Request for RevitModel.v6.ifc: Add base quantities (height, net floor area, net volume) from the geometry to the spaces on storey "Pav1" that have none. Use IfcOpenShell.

First a look at what the model holds.

```python
import ifcopenshell
import ifcopenshell.util.element
import ifcopenshell.util.unit

model = ifcopenshell.open("RevitModel.v6.ifc")
print(model.schema)
for unit_type in ("LENGTHUNIT", "AREAUNIT", "VOLUMEUNIT"):
    print(unit_type, ifcopenshell.util.unit.calculate_unit_scale(model, unit_type))
storey = next(s for s in model.by_type("IfcBuildingStorey") if s.Name == "Pav1")
spaces = [e for e in ifcopenshell.util.element.get_decomposition(storey) if e.is_a("IfcSpace")]
for e in sorted(spaces, key=lambda e: e.id()):
    print(e.id(), e.is_a(), e.Name, list(ifcopenshell.util.element.get_psets(e, qtos_only=True)), sep=" | ")
```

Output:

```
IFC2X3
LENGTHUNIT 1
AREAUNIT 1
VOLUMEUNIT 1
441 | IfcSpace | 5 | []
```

```python
import ifcopenshell
import ifcopenshell.api.pset
import ifcopenshell.geom
import ifcopenshell.util.element
import ifcopenshell.util.shape
import ifcopenshell.util.unit

model = ifcopenshell.open("RevitModel.v6.ifc")
unit_scale = ifcopenshell.util.unit.calculate_unit_scale(model)
area_scale = ifcopenshell.util.unit.calculate_unit_scale(model, "AREAUNIT")
volume_scale = ifcopenshell.util.unit.calculate_unit_scale(model, "VOLUMEUNIT")
settings = ifcopenshell.geom.settings()

storey = next(s for s in model.by_type("IfcBuildingStorey") if s.Name == "Pav1")
spaces = [e for e in ifcopenshell.util.element.get_decomposition(storey) if e.is_a("IfcSpace")]

for e in sorted(spaces, key=lambda e: e.id()):
    if ifcopenshell.util.element.get_psets(e, qtos_only=True, should_inherit=False):
        continue
    # Geometry comes back in metres, in the element's own axes.
    shape = ifcopenshell.geom.create_shape(settings, e)
    values = {
        "Height": ifcopenshell.util.shape.get_z(shape.geometry) / unit_scale,
        "NetFloorArea": ifcopenshell.util.shape.get_footprint_area(shape.geometry) / area_scale,
        "NetVolume": ifcopenshell.util.shape.get_volume(shape.geometry) / volume_scale,
    }
    qto = ifcopenshell.api.pset.add_qto(model, product=e, name="BaseQuantities")
    ifcopenshell.api.pset.edit_qto(model, qto=qto, properties=values)
    print(e.id(), {k: round(v, 3) for k, v in values.items()})

model.write("RevitModel.v6-out.ifc")
```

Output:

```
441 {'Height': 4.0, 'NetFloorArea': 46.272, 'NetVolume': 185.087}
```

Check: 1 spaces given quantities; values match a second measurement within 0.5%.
